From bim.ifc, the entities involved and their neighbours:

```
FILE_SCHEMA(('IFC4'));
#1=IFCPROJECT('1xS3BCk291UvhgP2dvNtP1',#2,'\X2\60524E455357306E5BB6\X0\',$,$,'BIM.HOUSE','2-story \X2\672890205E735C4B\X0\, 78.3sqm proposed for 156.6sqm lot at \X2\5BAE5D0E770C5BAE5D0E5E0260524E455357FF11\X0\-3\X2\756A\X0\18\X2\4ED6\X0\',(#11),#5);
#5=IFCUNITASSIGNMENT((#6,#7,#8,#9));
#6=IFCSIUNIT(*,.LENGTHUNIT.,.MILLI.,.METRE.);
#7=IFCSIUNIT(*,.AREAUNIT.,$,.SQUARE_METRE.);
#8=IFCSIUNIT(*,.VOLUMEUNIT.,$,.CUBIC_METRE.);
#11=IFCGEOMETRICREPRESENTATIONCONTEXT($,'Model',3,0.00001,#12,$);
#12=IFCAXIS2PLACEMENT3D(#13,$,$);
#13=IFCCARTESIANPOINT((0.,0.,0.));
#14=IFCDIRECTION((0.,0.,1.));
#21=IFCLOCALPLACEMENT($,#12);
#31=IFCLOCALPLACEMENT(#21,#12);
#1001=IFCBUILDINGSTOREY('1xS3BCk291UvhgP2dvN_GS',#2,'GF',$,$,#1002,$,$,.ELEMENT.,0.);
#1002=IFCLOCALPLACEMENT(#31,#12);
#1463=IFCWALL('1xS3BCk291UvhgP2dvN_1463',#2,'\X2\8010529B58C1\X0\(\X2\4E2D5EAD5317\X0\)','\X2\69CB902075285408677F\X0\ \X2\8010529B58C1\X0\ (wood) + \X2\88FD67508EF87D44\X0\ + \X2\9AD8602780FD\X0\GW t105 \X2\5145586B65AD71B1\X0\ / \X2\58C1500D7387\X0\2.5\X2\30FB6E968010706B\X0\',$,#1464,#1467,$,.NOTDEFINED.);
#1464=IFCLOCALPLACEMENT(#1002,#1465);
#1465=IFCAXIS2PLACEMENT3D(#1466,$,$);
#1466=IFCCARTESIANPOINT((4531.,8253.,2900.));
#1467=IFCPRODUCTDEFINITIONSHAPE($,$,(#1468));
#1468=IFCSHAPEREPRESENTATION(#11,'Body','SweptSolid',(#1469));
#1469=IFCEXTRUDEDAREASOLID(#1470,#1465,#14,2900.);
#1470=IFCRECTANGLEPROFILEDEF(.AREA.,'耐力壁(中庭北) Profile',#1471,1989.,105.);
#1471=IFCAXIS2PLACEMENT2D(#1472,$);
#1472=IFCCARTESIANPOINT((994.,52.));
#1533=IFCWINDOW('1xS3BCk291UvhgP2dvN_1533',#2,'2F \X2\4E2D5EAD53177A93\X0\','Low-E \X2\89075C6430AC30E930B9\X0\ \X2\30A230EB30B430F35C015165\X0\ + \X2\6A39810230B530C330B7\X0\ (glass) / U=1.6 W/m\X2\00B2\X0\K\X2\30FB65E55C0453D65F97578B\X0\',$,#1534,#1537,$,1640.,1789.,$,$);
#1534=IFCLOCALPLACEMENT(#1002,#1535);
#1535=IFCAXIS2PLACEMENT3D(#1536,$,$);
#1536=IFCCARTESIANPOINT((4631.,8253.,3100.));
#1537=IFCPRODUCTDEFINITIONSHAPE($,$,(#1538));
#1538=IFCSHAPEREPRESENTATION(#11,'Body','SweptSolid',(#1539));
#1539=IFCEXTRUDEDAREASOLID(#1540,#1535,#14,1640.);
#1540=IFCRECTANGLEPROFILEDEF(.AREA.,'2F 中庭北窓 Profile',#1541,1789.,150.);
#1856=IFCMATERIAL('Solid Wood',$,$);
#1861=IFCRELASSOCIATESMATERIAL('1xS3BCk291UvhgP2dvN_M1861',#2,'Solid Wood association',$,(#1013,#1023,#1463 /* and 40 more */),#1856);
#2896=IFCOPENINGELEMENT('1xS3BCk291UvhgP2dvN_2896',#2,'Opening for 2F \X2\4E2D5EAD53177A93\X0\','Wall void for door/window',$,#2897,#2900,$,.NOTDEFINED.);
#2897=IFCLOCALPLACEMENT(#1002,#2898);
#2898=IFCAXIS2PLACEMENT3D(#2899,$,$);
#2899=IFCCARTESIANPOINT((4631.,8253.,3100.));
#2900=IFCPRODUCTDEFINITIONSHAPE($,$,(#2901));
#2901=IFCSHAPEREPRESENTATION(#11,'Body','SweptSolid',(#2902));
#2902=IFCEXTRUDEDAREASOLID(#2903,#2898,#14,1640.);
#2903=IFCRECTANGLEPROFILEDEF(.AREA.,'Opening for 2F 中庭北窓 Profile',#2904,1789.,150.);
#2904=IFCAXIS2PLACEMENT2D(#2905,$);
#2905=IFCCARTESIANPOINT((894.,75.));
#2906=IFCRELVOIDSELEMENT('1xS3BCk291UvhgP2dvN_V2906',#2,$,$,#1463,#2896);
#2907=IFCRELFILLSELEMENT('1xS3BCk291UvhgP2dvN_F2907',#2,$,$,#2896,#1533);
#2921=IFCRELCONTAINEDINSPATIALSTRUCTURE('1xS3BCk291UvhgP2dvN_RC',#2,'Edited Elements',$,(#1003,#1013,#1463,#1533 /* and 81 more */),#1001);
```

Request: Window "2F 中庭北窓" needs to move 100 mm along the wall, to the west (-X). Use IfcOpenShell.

```python
import ifcopenshell
import ifcopenshell.api.geometry
import ifcopenshell.util.placement
import ifcopenshell.util.unit

model = ifcopenshell.open("bim.ifc")
unit_scale = ifcopenshell.util.unit.calculate_unit_scale(model)

window = model.by_guid("1xS3BCk291UvhgP2dvN_1533")
opening = window.FillsVoids[0].RelatingOpeningElement
wall = opening.VoidsElements[0].RelatingBuildingElement

wall_matrix = ifcopenshell.util.placement.get_local_placement(wall.ObjectPlacement)
shift = wall_matrix[:3, 0] * -0.1 / unit_scale
before = ifcopenshell.util.placement.get_local_placement(window.ObjectPlacement)[:3, 3].copy()

# The window is not placed relative to its opening, so move both.
for product in (opening, window):
    matrix = ifcopenshell.util.placement.get_local_placement(product.ObjectPlacement)
    matrix[:3, 3] += shift
    ifcopenshell.api.geometry.edit_object_placement(model, product=product, matrix=matrix, is_si=False)

after = ifcopenshell.util.placement.get_local_placement(window.ObjectPlacement)[:3, 3]
print("window moved by", (after - before).round(3) + 0.0)

model.write("bim_v2.ifc")
```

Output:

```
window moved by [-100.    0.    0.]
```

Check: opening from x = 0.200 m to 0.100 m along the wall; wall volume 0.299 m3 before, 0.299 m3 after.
